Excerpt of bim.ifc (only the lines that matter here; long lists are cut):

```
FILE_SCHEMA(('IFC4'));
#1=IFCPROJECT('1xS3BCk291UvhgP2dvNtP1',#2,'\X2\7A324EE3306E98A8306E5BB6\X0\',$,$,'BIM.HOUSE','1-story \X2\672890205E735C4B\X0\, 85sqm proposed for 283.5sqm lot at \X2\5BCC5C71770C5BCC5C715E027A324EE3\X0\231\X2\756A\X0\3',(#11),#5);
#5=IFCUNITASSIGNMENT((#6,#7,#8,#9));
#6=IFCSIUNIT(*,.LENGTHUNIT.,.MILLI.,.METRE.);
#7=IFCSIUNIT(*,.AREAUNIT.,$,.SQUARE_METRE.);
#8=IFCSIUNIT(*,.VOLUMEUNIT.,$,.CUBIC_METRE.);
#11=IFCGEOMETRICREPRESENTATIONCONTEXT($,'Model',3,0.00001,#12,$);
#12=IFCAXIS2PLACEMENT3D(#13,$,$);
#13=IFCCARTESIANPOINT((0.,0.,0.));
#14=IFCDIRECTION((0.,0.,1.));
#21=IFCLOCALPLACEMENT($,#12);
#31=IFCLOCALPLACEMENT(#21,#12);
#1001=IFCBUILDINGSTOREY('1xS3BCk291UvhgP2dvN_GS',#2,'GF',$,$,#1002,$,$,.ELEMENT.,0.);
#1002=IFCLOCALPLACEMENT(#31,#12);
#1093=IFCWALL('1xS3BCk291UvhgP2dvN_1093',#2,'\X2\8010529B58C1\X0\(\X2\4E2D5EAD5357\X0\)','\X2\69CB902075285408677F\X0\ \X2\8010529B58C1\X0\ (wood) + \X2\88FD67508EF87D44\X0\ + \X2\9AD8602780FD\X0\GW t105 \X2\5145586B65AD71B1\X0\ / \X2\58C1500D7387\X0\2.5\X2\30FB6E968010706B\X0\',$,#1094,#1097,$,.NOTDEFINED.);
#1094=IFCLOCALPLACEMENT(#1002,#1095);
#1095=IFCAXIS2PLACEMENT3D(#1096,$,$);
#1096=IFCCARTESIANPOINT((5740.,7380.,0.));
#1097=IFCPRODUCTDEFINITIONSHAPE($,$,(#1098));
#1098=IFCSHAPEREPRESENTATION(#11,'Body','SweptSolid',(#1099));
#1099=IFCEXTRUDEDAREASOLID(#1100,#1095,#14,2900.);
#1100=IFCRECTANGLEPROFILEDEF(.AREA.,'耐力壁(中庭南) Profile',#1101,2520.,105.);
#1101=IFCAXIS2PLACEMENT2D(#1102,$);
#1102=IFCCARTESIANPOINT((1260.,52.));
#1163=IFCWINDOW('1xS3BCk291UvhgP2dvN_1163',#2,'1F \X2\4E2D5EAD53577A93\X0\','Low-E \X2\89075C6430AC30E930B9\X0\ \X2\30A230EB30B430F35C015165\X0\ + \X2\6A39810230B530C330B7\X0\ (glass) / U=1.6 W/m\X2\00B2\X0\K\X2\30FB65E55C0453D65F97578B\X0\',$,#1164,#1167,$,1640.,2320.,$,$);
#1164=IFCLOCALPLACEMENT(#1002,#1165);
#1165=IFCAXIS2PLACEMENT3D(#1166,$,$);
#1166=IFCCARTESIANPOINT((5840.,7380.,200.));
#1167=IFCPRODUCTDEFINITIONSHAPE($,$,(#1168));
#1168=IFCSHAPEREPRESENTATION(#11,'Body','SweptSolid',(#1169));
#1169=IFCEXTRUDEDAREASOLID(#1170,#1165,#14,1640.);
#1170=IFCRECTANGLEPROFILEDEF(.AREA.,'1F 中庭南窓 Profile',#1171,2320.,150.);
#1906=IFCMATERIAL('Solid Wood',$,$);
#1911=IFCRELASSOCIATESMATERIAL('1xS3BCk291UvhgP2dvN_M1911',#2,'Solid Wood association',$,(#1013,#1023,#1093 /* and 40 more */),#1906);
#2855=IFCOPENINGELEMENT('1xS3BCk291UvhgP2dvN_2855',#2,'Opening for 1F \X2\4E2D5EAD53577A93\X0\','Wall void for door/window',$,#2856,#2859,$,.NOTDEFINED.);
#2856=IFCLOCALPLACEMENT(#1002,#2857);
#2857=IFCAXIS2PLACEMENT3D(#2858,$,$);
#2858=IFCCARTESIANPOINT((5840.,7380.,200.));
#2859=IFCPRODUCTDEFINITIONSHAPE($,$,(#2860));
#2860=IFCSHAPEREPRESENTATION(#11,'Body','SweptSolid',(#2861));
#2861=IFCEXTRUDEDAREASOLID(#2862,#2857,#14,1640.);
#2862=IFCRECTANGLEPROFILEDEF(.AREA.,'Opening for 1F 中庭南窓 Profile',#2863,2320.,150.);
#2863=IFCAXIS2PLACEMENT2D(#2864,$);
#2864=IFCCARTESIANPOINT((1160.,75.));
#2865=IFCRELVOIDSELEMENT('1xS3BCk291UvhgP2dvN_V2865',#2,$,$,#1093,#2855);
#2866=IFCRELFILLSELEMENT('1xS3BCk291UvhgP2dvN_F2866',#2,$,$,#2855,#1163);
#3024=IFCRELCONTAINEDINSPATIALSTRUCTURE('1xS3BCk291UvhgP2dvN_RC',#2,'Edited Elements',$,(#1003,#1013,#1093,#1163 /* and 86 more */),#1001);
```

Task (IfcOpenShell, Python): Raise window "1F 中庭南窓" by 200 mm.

```python
import numpy as np
import ifcopenshell
import ifcopenshell.api.geometry
import ifcopenshell.util.placement
import ifcopenshell.util.unit

model = ifcopenshell.open("bim.ifc")
unit_scale = ifcopenshell.util.unit.calculate_unit_scale(model)

window = model.by_id(1163)
opening = window.FillsVoids[0].RelatingOpeningElement
dz = 0.2 / unit_scale

shift = np.array([0.0, 0.0, dz])
# The window is not placed relative to its opening, so move both.
for product in (opening, window):
    matrix = ifcopenshell.util.placement.get_local_placement(product.ObjectPlacement)
    matrix[:3, 3] += shift
    ifcopenshell.api.geometry.edit_object_placement(model, product=product, matrix=matrix, is_si=False)

print(f"moved by {dz * unit_scale:+.3f} m")

model.write("bim-out.ifc")
```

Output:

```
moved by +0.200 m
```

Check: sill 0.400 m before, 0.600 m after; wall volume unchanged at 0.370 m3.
